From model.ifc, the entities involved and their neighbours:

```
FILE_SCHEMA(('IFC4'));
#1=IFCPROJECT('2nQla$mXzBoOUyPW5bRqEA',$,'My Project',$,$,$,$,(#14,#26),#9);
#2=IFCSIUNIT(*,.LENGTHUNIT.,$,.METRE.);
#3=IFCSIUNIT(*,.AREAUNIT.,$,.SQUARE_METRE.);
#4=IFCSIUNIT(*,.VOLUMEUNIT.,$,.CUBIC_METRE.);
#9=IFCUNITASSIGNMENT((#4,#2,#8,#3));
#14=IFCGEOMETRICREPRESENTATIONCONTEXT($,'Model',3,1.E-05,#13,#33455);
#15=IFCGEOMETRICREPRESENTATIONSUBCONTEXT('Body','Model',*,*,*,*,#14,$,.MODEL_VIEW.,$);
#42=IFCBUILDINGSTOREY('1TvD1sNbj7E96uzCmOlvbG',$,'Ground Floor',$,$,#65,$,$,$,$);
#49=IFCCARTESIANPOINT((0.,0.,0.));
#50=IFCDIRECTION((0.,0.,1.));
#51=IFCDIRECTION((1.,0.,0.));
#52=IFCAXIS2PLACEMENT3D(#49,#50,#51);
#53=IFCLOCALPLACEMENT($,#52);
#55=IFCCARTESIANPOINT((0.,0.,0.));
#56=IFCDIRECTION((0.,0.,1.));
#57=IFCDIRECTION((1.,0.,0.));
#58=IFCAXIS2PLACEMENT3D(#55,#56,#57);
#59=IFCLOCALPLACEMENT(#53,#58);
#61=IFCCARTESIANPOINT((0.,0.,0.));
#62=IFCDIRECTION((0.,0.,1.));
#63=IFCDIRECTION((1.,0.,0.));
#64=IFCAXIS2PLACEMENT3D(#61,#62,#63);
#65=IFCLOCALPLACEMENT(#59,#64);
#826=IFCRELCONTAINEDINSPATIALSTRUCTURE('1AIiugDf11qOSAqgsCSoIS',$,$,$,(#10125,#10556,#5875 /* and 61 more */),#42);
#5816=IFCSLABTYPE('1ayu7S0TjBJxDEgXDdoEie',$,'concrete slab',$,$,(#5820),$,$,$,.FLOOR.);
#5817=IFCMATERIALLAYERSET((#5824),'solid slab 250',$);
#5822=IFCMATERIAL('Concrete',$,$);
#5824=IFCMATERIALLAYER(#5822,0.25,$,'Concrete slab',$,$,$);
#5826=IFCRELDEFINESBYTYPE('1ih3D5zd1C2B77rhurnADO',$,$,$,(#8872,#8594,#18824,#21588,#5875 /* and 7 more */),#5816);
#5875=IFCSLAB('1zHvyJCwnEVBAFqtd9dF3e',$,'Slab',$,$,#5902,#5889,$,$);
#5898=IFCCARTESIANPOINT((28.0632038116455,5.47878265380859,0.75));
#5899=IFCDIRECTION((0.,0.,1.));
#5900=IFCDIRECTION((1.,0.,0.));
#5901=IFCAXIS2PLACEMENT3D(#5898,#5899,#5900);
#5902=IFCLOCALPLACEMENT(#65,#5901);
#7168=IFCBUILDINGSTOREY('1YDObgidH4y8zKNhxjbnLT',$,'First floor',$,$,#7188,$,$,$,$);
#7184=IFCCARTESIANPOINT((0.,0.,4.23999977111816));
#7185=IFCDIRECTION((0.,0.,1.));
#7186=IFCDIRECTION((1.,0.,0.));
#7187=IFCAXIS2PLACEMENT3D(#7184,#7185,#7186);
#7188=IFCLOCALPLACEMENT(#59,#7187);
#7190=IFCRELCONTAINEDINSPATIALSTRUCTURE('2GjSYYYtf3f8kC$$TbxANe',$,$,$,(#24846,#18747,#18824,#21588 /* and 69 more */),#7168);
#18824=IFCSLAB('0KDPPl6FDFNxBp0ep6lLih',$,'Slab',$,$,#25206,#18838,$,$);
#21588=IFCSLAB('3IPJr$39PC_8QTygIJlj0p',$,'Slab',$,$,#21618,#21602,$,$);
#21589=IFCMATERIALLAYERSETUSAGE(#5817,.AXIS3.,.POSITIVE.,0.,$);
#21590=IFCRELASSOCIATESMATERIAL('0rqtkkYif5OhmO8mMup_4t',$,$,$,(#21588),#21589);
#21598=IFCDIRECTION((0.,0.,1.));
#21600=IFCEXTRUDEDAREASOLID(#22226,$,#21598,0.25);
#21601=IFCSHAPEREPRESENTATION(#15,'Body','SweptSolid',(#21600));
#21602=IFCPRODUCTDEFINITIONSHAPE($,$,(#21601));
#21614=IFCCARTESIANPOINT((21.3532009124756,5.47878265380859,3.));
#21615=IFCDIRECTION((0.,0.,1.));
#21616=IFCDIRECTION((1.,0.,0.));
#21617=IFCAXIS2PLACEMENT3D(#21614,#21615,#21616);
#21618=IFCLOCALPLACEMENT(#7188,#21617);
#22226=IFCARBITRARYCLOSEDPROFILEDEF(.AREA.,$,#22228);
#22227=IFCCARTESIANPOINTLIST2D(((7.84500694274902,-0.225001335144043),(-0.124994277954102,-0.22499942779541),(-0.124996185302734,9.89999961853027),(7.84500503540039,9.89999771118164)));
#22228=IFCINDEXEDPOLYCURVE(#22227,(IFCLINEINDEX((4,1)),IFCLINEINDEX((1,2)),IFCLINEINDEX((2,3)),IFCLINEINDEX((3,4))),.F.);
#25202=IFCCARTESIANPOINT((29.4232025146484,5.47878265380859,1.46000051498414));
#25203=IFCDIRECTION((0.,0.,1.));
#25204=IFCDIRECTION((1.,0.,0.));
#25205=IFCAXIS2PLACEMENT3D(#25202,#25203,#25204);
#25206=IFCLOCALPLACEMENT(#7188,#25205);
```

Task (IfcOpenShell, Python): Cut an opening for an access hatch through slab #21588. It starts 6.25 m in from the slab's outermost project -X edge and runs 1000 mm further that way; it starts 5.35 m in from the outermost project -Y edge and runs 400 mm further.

```python
import numpy as np
import ifcopenshell
import ifcopenshell.api.feature
import ifcopenshell.api.geometry
import ifcopenshell.api.root
import ifcopenshell.geom
import ifcopenshell.util.placement
import ifcopenshell.util.representation
import ifcopenshell.util.shape
import ifcopenshell.util.unit

model = ifcopenshell.open("model.ifc")
unit_scale = ifcopenshell.util.unit.calculate_unit_scale(model)
settings = ifcopenshell.geom.settings()


def volume(element):
    """Net volume in cubic metres, openings subtracted."""
    shape = ifcopenshell.geom.create_shape(settings, element)
    return ifcopenshell.util.shape.get_volume(shape.geometry)


slab = model.by_guid("3IPJr$39PC_8QTygIJlj0p")
before = volume(slab)

# Extent in the slab's own axes, in metres. The edges named are its -X and -Y sides.
slab_shape = ifcopenshell.geom.create_shape(settings, slab)
vertices = ifcopenshell.util.shape.get_vertices(slab_shape.geometry)
x_min, y_min, bottom = vertices.min(axis=0)
top = vertices[:, 2].max()

opening = ifcopenshell.api.root.create_entity(model, ifc_class="IfcOpeningElement", name="Access hatch opening", predefined_type="OPENING")
context = ifcopenshell.util.representation.get_context(model, "Model", "Body", "MODEL_VIEW")
width, depth = 1, 0.4
outline = [(0.0, 0.0), (width, 0.0), (width, depth), (0.0, depth), (0.0, 0.0)]
# Overshoot both faces by 50 mm so the cut is clean.
shape = ifcopenshell.api.geometry.add_slab_representation(
    model, context=context, depth=top - bottom + 0.1, polyline=outline
)
ifcopenshell.api.geometry.assign_representation(model, product=opening, representation=shape)

matrix = ifcopenshell.util.placement.get_local_placement(slab.ObjectPlacement)
matrix[:, 3] = matrix @ np.append(np.array([x_min + 6.25, y_min + 5.35, bottom - 0.05]) / unit_scale, 1.0)
ifcopenshell.api.geometry.edit_object_placement(model, product=opening, matrix=matrix, is_si=False)
ifcopenshell.api.feature.add_feature(model, feature=opening, element=slab)

after = volume(slab)

print(f"slab volume {before:.3f} -> {after:.3f} m3")

model.write("model_rev.ifc")
```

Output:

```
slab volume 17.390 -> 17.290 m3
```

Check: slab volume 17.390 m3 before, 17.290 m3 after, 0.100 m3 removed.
